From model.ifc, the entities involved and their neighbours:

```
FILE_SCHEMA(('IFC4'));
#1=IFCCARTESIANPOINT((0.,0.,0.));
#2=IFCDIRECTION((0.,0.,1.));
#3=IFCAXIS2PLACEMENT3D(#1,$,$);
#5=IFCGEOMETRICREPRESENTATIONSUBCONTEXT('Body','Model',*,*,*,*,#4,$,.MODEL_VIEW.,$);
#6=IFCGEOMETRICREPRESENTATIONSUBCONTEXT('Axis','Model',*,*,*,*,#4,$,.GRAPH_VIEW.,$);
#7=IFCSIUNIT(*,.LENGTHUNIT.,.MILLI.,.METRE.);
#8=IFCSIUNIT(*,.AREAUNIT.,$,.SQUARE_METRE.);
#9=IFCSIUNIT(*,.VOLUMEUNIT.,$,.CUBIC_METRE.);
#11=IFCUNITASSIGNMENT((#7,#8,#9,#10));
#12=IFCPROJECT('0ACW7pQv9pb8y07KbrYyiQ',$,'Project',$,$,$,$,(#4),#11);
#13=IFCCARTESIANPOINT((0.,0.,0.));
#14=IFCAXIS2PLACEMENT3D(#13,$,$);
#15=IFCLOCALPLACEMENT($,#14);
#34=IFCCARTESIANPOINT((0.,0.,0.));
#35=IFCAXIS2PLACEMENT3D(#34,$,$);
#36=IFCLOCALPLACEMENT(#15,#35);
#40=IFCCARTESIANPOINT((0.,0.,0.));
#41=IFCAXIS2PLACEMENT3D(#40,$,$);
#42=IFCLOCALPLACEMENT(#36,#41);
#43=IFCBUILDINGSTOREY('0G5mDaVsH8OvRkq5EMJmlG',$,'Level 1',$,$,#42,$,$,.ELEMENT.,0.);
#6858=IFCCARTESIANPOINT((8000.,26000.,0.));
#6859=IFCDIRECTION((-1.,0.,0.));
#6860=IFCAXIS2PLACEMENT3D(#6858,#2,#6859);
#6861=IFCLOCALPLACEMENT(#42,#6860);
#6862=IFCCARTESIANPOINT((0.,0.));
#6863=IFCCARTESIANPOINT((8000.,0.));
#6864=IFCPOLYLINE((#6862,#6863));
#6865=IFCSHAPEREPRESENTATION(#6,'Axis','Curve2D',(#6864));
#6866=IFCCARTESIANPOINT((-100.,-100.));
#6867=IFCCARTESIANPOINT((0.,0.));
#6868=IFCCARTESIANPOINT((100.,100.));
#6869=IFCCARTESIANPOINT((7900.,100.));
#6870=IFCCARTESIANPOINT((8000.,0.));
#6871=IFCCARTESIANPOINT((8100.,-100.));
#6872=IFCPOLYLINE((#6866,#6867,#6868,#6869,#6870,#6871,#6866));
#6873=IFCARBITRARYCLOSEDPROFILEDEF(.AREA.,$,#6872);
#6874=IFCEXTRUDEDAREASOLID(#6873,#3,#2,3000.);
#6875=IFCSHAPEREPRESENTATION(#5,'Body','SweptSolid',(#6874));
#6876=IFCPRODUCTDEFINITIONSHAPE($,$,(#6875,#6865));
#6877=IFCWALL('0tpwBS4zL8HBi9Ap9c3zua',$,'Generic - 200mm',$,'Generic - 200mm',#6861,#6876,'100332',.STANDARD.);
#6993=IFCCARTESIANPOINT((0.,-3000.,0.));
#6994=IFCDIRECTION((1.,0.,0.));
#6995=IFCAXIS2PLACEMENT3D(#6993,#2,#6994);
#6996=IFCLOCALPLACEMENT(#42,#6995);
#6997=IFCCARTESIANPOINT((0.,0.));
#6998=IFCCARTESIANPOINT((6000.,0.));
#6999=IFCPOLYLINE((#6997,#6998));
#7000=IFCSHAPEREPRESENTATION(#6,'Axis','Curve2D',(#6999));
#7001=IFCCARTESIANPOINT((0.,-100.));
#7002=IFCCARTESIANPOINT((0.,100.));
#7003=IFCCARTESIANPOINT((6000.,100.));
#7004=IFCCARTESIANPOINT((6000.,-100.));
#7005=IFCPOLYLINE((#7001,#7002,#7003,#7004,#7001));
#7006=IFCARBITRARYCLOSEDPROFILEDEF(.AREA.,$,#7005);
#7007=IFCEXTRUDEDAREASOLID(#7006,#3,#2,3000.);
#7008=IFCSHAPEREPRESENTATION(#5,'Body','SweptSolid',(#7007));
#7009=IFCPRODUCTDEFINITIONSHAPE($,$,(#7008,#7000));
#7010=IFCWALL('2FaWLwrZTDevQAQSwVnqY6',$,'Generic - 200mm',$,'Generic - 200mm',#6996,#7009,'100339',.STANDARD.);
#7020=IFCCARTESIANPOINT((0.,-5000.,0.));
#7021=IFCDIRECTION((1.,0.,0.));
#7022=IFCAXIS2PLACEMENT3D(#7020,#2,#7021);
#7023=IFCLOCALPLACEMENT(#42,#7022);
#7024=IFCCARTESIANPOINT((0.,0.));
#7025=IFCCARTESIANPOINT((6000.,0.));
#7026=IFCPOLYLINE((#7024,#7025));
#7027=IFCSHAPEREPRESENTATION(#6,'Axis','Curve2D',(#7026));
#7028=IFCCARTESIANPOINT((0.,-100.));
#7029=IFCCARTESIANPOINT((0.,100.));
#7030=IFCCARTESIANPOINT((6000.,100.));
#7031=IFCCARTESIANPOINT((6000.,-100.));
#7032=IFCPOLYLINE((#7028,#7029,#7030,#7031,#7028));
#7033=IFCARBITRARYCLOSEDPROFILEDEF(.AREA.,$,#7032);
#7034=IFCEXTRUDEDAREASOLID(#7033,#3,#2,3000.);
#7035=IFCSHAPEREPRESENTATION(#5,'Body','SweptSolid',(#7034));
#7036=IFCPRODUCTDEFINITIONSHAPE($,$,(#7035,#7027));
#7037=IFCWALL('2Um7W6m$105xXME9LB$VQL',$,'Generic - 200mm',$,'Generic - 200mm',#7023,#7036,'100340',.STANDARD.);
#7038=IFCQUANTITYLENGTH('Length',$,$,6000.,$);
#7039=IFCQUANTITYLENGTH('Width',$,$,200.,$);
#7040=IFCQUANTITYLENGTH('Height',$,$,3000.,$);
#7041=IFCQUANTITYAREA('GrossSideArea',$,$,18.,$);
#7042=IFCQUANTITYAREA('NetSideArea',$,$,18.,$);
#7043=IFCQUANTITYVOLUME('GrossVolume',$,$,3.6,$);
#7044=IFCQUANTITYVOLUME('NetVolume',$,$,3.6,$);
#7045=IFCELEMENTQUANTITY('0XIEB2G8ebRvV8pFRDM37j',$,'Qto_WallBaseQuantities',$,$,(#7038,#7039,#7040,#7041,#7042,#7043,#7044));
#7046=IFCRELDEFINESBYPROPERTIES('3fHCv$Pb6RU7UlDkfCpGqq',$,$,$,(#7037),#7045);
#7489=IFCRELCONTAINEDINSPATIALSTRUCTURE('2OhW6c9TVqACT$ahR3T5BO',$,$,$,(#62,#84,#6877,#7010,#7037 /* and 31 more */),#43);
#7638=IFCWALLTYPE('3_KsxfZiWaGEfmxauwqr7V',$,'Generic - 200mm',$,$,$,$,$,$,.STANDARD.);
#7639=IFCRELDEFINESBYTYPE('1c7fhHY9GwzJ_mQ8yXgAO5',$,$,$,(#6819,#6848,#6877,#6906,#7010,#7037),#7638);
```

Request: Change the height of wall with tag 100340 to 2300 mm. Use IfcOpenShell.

```python
import ifcopenshell
import ifcopenshell.api.pset
import ifcopenshell.geom
import ifcopenshell.util.element
import ifcopenshell.util.representation
import ifcopenshell.util.shape
import ifcopenshell.util.unit

model = ifcopenshell.open("model.ifc")
unit_scale = ifcopenshell.util.unit.calculate_unit_scale(model)
area_scale = ifcopenshell.util.unit.calculate_unit_scale(model, "AREAUNIT")
volume_scale = ifcopenshell.util.unit.calculate_unit_scale(model, "VOLUMEUNIT")
settings = ifcopenshell.geom.settings()


def volume(element):
    """Net volume in cubic metres, openings subtracted."""
    shape = ifcopenshell.geom.create_shape(settings, element)
    return ifcopenshell.util.shape.get_volume(shape.geometry)


wall = model.by_guid("2Um7W6m$105xXME9LB$VQL")
before = volume(wall)

body = ifcopenshell.util.representation.get_representation(wall, "Model", "Body")
solid = body.Items[0]
old_height = solid.Depth
solid.Depth = 2.3 / unit_scale
after = volume(wall)
thickness = 0.2  # wall thickness in metres

# Update the stored height, areas and volumes.
qto = model.by_id(ifcopenshell.util.element.get_pset(wall, "Qto_WallBaseQuantities", should_inherit=False)["id"])
ifcopenshell.api.pset.edit_qto(model, qto=qto, properties={
    "Height": solid.Depth,
    "GrossSideArea": ifcopenshell.util.element.get_pset(wall, "Qto_WallBaseQuantities", "GrossSideArea") * solid.Depth / old_height,
    "NetSideArea": after / thickness / area_scale,
    "GrossVolume": ifcopenshell.util.element.get_pset(wall, "Qto_WallBaseQuantities", "GrossVolume") * solid.Depth / old_height,
    "NetVolume": after / volume_scale,
})

print(f"height {old_height:g} -> {solid.Depth:g}, volume {before:.3f} -> {after:.3f} m3")

model.write("model_v2.ifc")
```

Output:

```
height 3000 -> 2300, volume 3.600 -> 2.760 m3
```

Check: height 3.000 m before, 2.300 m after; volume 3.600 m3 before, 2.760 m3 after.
